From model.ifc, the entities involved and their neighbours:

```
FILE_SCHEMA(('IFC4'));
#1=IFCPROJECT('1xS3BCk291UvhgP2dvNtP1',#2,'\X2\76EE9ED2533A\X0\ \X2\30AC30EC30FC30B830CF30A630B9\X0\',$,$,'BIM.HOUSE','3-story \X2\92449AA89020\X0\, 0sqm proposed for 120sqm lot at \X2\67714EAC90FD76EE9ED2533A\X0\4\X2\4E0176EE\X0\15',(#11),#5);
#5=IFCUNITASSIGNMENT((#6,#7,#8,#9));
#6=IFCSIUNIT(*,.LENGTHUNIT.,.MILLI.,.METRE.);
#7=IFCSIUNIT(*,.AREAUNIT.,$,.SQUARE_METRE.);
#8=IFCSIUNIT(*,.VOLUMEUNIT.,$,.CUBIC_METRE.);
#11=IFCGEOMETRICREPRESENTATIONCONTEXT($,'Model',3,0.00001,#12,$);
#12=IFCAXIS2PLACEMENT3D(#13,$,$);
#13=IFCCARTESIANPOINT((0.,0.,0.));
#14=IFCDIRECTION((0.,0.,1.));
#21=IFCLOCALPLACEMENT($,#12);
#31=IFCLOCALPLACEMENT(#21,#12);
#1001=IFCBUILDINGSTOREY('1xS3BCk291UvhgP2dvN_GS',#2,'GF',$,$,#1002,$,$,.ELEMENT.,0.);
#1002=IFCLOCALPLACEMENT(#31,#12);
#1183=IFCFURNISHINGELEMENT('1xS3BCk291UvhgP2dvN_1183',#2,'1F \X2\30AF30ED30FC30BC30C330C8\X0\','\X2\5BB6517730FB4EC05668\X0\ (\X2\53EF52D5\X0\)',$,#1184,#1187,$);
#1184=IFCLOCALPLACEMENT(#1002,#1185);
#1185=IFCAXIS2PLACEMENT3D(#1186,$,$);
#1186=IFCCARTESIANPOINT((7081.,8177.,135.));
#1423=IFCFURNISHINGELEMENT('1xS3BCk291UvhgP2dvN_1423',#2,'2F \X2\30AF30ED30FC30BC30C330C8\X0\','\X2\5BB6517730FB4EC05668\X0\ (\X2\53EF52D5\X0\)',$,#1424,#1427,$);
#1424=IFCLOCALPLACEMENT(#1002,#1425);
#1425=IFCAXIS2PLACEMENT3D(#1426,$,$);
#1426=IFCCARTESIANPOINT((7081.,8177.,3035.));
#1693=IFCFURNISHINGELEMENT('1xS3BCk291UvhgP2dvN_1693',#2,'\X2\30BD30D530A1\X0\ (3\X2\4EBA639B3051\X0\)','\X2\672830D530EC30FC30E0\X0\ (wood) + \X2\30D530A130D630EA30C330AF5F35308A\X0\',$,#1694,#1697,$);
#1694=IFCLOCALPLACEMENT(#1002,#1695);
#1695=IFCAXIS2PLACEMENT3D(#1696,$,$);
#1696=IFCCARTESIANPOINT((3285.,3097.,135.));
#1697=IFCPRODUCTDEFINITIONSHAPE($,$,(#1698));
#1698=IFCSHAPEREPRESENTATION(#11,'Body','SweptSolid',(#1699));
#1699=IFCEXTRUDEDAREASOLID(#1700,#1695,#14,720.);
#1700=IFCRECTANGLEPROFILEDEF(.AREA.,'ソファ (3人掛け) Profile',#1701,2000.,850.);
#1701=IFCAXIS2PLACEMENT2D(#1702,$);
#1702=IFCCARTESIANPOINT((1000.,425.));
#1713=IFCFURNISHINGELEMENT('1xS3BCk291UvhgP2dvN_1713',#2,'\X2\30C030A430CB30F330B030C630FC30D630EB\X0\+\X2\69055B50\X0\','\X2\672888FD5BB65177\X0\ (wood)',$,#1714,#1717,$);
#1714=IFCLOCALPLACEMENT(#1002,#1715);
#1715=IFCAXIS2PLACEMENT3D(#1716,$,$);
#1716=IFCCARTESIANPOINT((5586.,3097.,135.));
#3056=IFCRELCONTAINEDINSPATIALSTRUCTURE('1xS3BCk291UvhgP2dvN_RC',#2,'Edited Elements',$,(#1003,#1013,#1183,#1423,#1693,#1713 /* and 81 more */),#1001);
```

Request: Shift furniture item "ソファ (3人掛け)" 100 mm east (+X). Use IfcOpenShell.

```python
import ifcopenshell
import ifcopenshell.api.geometry
import ifcopenshell.util.placement
import ifcopenshell.util.unit

model = ifcopenshell.open("model.ifc")
unit_scale = ifcopenshell.util.unit.calculate_unit_scale(model)

item = model.by_guid("1xS3BCk291UvhgP2dvN_1693")
matrix = ifcopenshell.util.placement.get_local_placement(item.ObjectPlacement)
matrix[0, 3] += 0.1 / unit_scale
ifcopenshell.api.geometry.edit_object_placement(model, product=item, matrix=matrix, is_si=False)

print(ifcopenshell.util.placement.get_local_placement(item.ObjectPlacement).round(3) + 0.0)

model.write("model-out.ifc")
```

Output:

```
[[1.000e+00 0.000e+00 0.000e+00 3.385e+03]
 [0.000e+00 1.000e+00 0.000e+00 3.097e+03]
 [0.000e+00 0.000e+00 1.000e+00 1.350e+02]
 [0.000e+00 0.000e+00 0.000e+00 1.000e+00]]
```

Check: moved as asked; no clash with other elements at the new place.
